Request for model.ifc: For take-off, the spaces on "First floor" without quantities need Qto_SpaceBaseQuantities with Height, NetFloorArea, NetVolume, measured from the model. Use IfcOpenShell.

First a look at what the model holds.

```python
import ifcopenshell
import ifcopenshell.util.element
import ifcopenshell.util.unit

model = ifcopenshell.open("model.ifc")
print(model.schema)
for unit_type in ("LENGTHUNIT", "AREAUNIT", "VOLUMEUNIT"):
    print(unit_type, ifcopenshell.util.unit.calculate_unit_scale(model, unit_type))
storey = next(s for s in model.by_type("IfcBuildingStorey") if s.Name == "First floor")
spaces = [e for e in ifcopenshell.util.element.get_decomposition(storey) if e.is_a("IfcSpace")]
for e in sorted(spaces, key=lambda e: e.id()):
    print(e.id(), e.is_a(), e.Name, list(ifcopenshell.util.element.get_psets(e, qtos_only=True)), sep=" | ")
```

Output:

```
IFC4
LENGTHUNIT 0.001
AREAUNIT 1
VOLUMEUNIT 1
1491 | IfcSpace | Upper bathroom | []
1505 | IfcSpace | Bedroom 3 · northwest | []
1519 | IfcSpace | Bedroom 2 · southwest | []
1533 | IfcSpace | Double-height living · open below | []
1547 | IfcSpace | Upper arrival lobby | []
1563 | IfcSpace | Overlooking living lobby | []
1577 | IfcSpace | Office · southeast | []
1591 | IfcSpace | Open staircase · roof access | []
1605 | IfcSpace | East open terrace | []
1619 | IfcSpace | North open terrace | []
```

```python
import ifcopenshell
import ifcopenshell.api.pset
import ifcopenshell.geom
import ifcopenshell.util.element
import ifcopenshell.util.shape
import ifcopenshell.util.unit

model = ifcopenshell.open("model.ifc")
unit_scale = ifcopenshell.util.unit.calculate_unit_scale(model)
area_scale = ifcopenshell.util.unit.calculate_unit_scale(model, "AREAUNIT")
volume_scale = ifcopenshell.util.unit.calculate_unit_scale(model, "VOLUMEUNIT")
settings = ifcopenshell.geom.settings()

storey = next(s for s in model.by_type("IfcBuildingStorey") if s.Name == "First floor")
spaces = [e for e in ifcopenshell.util.element.get_decomposition(storey) if e.is_a("IfcSpace")]

for e in sorted(spaces, key=lambda e: e.id()):
    if ifcopenshell.util.element.get_psets(e, qtos_only=True, should_inherit=False):
        continue
    # Geometry comes back in metres, in the element's own axes.
    shape = ifcopenshell.geom.create_shape(settings, e)
    values = {
        "Height": ifcopenshell.util.shape.get_z(shape.geometry) / unit_scale,
        "NetFloorArea": ifcopenshell.util.shape.get_footprint_area(shape.geometry) / area_scale,
        "NetVolume": ifcopenshell.util.shape.get_volume(shape.geometry) / volume_scale,
    }
    qto = ifcopenshell.api.pset.add_qto(model, product=e, name="Qto_SpaceBaseQuantities")
    ifcopenshell.api.pset.edit_qto(model, qto=qto, properties=values)
    print(e.id(), {k: round(v, 3) for k, v in values.items()})

model.write("model_edited.ifc")
```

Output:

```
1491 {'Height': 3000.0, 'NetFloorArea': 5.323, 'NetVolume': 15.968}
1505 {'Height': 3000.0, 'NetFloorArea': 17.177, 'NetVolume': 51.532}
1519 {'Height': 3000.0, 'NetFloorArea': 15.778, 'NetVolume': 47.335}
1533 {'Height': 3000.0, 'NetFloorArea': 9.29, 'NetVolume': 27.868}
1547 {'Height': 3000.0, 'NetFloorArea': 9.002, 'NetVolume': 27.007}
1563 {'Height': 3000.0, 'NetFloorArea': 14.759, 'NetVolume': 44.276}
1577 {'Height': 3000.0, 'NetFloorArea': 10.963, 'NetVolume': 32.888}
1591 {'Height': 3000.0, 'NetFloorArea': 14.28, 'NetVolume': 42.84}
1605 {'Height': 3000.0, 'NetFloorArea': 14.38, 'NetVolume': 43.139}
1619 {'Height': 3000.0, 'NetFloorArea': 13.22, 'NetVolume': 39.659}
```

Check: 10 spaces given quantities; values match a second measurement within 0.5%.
